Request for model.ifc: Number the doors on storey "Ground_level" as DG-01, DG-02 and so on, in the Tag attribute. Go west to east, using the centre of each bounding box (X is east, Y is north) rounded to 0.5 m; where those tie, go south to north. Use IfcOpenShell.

First a look at what the model holds.

```python
import ifcopenshell
import ifcopenshell.util.element
import ifcopenshell.util.placement

model = ifcopenshell.open("model.ifc")
print(model.schema)
storey = next(s for s in model.by_type("IfcBuildingStorey") if s.Name == "Ground_level")
doors = [e for e in ifcopenshell.util.element.get_decomposition(storey) if e.is_a("IfcDoor")]
for e in sorted(doors, key=lambda e: e.id()):
    origin = ifcopenshell.util.placement.get_local_placement(e.ObjectPlacement)[:3, 3]
    print(e.id(), e.Tag, e.Name, origin.round(2) + 0.0, sep=" | ")
```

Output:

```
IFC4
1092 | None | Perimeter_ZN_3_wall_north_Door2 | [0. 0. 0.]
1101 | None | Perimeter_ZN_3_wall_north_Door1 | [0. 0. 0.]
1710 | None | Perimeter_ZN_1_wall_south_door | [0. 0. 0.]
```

```python
import ifcopenshell
import ifcopenshell.geom
import ifcopenshell.util.element
import ifcopenshell.util.shape

model = ifcopenshell.open("model.ifc")
settings = ifcopenshell.geom.settings()
settings.set("use-world-coords", True)


def centre(element):
    shape = ifcopenshell.geom.create_shape(settings, element)
    return ifcopenshell.util.shape.get_bbox_centroid(shape.geometry)


storey = next(s for s in model.by_type("IfcBuildingStorey") if s.Name == "Ground_level")
doors = [e for e in ifcopenshell.util.element.get_decomposition(storey) if e.is_a("IfcDoor")]

# Insertion points can sit at a corner or the storey origin, so sort by the geometry (in metres).
centres = {e: centre(e) for e in doors}
doors.sort(key=lambda e: (round(centres[e][0] / 0.5), centres[e][1]))

for i, e in enumerate(doors, start=1):
    number = f"DG-{i:02d}"
    e.Tag = number
    print(e.id(), number)

model.write("model_updated.ifc")
```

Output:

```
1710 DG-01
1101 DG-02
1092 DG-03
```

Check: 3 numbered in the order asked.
